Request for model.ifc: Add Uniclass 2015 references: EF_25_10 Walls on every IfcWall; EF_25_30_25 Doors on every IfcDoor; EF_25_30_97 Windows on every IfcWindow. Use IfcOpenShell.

First a look at what the model holds.

```python
import ifcopenshell

model = ifcopenshell.open("model.ifc")
print(model.schema)
print("classifications:", [c.Name for c in model.by_type("IfcClassification")])
for ifc_class in ("IfcDoor", "IfcRoof", "IfcStair", "IfcWall", "IfcWindow"):
    print(ifc_class, len(model.by_type(ifc_class)))
```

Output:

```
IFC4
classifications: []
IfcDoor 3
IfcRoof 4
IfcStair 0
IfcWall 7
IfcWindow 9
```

```python
import ifcopenshell
import ifcopenshell.api.classification

model = ifcopenshell.open("model.ifc")

system = ifcopenshell.api.classification.add_classification(model, classification="Uniclass 2015")

codes = {
    "IfcWall": ("EF_25_10", "Walls"),
    "IfcDoor": ("EF_25_30_25", "Doors"),
    "IfcWindow": ("EF_25_30_97", "Windows"),
}
for ifc_class, (code, name) in codes.items():
    products = model.by_type(ifc_class)
    ifcopenshell.api.classification.add_reference(
        model, products=products, classification=system, identification=code, name=name
    )
    print(code, len(products))

model.write("model-out.ifc")
```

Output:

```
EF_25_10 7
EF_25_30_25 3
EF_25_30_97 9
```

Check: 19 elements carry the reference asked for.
